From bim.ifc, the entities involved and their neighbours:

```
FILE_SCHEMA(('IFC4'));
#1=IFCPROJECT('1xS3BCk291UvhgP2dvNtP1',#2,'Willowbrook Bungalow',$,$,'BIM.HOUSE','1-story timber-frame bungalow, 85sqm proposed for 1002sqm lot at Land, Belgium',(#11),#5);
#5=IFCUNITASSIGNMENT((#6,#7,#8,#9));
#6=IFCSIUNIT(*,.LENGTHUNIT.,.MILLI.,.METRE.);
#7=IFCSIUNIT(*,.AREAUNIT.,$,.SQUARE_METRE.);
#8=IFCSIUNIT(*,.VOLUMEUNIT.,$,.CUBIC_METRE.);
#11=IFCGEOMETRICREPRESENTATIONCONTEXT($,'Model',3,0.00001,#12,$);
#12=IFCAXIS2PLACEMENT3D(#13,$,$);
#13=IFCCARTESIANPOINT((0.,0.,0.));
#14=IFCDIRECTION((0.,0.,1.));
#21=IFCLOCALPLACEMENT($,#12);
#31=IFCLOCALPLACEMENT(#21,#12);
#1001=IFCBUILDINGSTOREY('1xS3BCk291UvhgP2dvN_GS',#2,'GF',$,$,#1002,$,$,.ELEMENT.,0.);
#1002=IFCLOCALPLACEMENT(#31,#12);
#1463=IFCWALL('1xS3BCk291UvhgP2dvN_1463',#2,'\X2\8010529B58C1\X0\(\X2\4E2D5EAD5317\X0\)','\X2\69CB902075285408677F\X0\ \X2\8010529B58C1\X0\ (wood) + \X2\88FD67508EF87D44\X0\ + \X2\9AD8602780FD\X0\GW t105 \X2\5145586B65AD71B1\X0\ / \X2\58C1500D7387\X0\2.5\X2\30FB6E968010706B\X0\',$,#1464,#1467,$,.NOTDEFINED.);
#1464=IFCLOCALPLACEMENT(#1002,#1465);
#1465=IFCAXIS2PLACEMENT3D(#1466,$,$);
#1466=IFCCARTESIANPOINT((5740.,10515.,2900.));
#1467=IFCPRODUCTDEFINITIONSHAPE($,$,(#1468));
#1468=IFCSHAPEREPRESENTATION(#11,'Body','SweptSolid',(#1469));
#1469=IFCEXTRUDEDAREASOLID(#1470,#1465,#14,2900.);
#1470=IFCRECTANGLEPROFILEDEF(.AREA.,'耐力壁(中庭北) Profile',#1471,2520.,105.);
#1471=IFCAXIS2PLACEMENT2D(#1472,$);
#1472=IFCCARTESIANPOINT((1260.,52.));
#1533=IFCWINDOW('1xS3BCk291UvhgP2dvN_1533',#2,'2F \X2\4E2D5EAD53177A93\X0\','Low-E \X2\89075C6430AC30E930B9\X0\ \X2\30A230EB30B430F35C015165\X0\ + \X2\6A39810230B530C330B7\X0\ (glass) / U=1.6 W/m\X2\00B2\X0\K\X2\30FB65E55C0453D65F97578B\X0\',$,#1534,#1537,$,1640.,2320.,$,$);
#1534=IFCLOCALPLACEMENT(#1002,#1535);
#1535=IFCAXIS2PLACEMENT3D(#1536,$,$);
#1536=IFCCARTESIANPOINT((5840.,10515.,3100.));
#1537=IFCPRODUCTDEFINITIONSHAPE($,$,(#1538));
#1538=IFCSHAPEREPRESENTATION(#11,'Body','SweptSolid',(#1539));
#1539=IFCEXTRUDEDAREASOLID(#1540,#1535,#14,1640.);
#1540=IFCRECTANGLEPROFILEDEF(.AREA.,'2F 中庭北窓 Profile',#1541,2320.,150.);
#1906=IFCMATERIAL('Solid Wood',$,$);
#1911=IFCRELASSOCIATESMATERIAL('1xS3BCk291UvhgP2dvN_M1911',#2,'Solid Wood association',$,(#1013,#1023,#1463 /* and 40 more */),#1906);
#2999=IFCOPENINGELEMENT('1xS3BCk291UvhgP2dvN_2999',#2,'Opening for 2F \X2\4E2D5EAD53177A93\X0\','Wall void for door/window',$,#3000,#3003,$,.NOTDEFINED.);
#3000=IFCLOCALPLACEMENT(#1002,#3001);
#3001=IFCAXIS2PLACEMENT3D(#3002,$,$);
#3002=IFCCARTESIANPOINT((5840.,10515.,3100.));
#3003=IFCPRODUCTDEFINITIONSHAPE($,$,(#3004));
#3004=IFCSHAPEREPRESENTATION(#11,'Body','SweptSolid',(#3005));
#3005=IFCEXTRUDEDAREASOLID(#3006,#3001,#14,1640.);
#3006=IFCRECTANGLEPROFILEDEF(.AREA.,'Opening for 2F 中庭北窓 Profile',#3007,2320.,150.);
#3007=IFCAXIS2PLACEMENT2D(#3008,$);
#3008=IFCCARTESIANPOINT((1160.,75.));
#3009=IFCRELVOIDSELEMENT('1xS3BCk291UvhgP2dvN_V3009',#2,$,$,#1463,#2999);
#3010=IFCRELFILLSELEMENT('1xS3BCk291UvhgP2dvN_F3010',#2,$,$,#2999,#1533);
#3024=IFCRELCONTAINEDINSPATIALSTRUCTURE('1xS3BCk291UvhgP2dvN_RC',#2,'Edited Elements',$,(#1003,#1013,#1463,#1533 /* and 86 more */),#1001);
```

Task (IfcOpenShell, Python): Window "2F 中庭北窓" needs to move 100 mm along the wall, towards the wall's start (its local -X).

```python
import ifcopenshell
import ifcopenshell.api.geometry
import ifcopenshell.util.placement

model = ifcopenshell.open("bim.ifc")

window = model.by_guid("1xS3BCk291UvhgP2dvN_1533")
opening = window.FillsVoids[0].RelatingOpeningElement
wall = opening.VoidsElements[0].RelatingBuildingElement

wall_matrix = ifcopenshell.util.placement.get_local_placement(wall.ObjectPlacement)
shift = wall_matrix[:3, 0] * -100.0
before = ifcopenshell.util.placement.get_local_placement(window.ObjectPlacement)[:3, 3].copy()

# The window is not placed relative to its opening, so move both.
for product in (opening, window):
    matrix = ifcopenshell.util.placement.get_local_placement(product.ObjectPlacement)
    matrix[:3, 3] += shift
    ifcopenshell.api.geometry.edit_object_placement(model, product=product, matrix=matrix, is_si=False)

after = ifcopenshell.util.placement.get_local_placement(window.ObjectPlacement)[:3, 3]
print("window moved by", (after - before).round(3) + 0.0)

model.write("bim_edited.ifc")
```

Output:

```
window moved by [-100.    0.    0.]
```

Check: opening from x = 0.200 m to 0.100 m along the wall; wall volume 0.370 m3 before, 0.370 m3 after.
